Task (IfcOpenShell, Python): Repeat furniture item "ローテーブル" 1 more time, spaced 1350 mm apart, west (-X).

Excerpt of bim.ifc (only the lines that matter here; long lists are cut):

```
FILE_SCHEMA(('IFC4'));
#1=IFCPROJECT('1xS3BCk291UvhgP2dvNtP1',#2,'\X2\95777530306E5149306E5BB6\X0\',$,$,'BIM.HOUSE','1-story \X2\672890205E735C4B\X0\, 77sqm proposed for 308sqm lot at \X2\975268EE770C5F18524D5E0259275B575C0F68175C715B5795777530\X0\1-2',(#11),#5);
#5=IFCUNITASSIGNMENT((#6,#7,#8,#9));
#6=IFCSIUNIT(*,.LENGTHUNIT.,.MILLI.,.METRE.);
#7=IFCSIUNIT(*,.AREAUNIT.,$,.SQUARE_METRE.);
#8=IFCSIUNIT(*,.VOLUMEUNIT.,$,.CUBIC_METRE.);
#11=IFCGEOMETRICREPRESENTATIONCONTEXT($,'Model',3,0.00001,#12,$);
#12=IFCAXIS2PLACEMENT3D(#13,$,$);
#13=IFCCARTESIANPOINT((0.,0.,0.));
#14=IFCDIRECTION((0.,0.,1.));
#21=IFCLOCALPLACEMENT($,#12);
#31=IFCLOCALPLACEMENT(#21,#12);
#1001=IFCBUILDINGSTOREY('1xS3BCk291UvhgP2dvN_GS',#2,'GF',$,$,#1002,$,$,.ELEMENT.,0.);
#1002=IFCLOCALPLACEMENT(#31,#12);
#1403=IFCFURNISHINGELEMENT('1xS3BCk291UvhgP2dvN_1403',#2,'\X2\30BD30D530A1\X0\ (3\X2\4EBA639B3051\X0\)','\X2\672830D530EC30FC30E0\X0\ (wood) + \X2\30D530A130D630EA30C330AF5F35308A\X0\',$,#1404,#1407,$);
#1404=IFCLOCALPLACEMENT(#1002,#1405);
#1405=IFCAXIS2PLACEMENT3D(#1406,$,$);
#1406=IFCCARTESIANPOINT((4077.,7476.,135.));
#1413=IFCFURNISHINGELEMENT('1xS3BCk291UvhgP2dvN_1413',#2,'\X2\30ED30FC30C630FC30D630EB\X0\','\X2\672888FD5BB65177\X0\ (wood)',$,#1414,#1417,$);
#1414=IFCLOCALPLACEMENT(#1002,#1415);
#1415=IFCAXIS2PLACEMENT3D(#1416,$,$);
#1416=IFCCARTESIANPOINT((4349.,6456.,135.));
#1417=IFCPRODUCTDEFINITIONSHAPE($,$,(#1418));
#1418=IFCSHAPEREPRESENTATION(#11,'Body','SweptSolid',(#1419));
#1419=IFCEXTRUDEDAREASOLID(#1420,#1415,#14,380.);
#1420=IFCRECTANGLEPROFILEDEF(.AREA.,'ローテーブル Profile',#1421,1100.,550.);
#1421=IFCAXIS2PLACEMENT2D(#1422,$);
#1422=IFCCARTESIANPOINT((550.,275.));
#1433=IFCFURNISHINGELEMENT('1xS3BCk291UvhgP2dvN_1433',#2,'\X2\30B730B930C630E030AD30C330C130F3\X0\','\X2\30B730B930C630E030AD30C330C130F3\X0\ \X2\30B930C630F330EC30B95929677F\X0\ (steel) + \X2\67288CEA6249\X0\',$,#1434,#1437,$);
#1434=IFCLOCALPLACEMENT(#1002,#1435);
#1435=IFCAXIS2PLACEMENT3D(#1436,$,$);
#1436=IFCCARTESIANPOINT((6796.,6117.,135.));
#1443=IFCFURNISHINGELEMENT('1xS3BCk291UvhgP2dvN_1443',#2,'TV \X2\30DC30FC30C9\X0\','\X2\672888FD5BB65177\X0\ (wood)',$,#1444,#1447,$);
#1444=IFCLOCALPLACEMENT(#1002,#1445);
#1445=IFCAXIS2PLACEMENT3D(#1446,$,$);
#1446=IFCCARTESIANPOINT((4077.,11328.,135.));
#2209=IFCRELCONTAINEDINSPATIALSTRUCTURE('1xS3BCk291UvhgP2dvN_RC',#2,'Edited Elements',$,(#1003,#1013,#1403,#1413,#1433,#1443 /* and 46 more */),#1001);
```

```python
import numpy as np
import ifcopenshell
import ifcopenshell.api.geometry
import ifcopenshell.api.root
import ifcopenshell.util.element
import ifcopenshell.util.placement
import ifcopenshell.util.unit

model = ifcopenshell.open("bim.ifc")
unit_scale = ifcopenshell.util.unit.calculate_unit_scale(model)


def reuse_history(source, copy):
    """copy_class also copies each property set's owner history, people and application; keep the originals."""
    for rel in copy.IsDefinedBy:
        if rel.is_a("IfcRelDefinesByProperties") and (history := rel.RelatingPropertyDefinition.OwnerHistory):
            rel.RelatingPropertyDefinition.OwnerHistory = source.OwnerHistory
            ifcopenshell.util.element.remove_deep2(model, history)


source = model.by_guid("1xS3BCk291UvhgP2dvN_1413")
base = ifcopenshell.util.placement.get_local_placement(source.ObjectPlacement)
step = np.array([-1.0, 0.0, 0.0]) * 1.35 / unit_scale

for i in range(1, 2):
    copy = ifcopenshell.api.root.copy_class(model, product=source)
    copy.Representation = ifcopenshell.util.element.copy_deep(
        model, source.Representation, exclude=["IfcGeometricRepresentationContext", "IfcRepresentationMap"]
    )
    reuse_history(source, copy)
    matrix = base.copy()
    matrix[:3, 3] += i * step
    print("added at", matrix[:3, 3].round(3) + 0.0)
    ifcopenshell.api.geometry.edit_object_placement(model, product=copy, matrix=matrix, is_si=False)

model.write("bim_edited.ifc")
```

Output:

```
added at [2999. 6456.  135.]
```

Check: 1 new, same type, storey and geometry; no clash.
